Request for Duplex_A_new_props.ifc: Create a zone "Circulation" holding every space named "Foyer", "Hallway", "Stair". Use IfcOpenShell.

First a look at what the model holds.

```python
import ifcopenshell

model = ifcopenshell.open("Duplex_A_new_props.ifc")
print(model.schema)
seen = {}
for space in model.by_type("IfcSpace"):
    seen[space.LongName] = seen.get(space.LongName, 0) + 1
for name, count in sorted(seen.items(), key=str):
    print(count, "x", name)
print("zones:", [z.Name for z in model.by_type("IfcZone")][:20])
```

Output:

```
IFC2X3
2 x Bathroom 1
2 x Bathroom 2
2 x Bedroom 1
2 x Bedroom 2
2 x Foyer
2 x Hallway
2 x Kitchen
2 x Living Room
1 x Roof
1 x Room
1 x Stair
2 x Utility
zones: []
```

```python
import ifcopenshell
import ifcopenshell.api.group
import ifcopenshell.api.root

model = ifcopenshell.open("Duplex_A_new_props.ifc")

names = {"Foyer", "Hallway", "Stair"}
spaces = [s for s in model.by_type("IfcSpace") if s.LongName in names]

zone = ifcopenshell.api.root.create_entity(model, ifc_class="IfcZone", name="Circulation")
ifcopenshell.api.group.assign_group(model, products=spaces, group=zone)
print(len(spaces), "spaces in", zone.Name)

model.write("Duplex_A_new_props_rev.ifc")
```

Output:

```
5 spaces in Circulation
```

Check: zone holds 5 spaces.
